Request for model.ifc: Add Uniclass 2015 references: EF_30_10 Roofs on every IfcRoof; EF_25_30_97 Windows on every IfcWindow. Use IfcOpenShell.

First a look at what the model holds.

```python
import ifcopenshell

model = ifcopenshell.open("model.ifc")
print(model.schema)
print("classifications:", [c.Name for c in model.by_type("IfcClassification")])
for ifc_class in ("IfcDoor", "IfcRoof", "IfcStair", "IfcWall", "IfcWindow"):
    print(ifc_class, len(model.by_type(ifc_class)))
```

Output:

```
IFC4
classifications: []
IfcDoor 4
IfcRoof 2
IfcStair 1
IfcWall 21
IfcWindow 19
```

```python
import ifcopenshell
import ifcopenshell.api.classification

model = ifcopenshell.open("model.ifc")

system = ifcopenshell.api.classification.add_classification(model, classification="Uniclass 2015")

codes = {
    "IfcRoof": ("EF_30_10", "Roofs"),
    "IfcWindow": ("EF_25_30_97", "Windows"),
}
for ifc_class, (code, name) in codes.items():
    products = model.by_type(ifc_class)
    ifcopenshell.api.classification.add_reference(
        model, products=products, classification=system, identification=code, name=name
    )
    print(code, len(products))

model.write("model-out.ifc")
```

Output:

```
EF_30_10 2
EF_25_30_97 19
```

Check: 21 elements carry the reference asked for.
